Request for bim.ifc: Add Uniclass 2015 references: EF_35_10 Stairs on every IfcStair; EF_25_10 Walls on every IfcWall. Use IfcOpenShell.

First a look at what the model holds.

```python
import ifcopenshell

model = ifcopenshell.open("bim.ifc")
print(model.schema)
print("classifications:", [c.Name for c in model.by_type("IfcClassification")])
for ifc_class in ("IfcDoor", "IfcRoof", "IfcStair", "IfcWall", "IfcWindow"):
    print(ifc_class, len(model.by_type(ifc_class)))
```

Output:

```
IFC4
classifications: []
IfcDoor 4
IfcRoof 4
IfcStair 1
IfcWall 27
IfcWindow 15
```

```python
import ifcopenshell
import ifcopenshell.api.classification

model = ifcopenshell.open("bim.ifc")

system = ifcopenshell.api.classification.add_classification(model, classification="Uniclass 2015")

codes = {
    "IfcStair": ("EF_35_10", "Stairs"),
    "IfcWall": ("EF_25_10", "Walls"),
}
for ifc_class, (code, name) in codes.items():
    products = model.by_type(ifc_class)
    ifcopenshell.api.classification.add_reference(
        model, products=products, classification=system, identification=code, name=name
    )
    print(code, len(products))

model.write("bim-out.ifc")
```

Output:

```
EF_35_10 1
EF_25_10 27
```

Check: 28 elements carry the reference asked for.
